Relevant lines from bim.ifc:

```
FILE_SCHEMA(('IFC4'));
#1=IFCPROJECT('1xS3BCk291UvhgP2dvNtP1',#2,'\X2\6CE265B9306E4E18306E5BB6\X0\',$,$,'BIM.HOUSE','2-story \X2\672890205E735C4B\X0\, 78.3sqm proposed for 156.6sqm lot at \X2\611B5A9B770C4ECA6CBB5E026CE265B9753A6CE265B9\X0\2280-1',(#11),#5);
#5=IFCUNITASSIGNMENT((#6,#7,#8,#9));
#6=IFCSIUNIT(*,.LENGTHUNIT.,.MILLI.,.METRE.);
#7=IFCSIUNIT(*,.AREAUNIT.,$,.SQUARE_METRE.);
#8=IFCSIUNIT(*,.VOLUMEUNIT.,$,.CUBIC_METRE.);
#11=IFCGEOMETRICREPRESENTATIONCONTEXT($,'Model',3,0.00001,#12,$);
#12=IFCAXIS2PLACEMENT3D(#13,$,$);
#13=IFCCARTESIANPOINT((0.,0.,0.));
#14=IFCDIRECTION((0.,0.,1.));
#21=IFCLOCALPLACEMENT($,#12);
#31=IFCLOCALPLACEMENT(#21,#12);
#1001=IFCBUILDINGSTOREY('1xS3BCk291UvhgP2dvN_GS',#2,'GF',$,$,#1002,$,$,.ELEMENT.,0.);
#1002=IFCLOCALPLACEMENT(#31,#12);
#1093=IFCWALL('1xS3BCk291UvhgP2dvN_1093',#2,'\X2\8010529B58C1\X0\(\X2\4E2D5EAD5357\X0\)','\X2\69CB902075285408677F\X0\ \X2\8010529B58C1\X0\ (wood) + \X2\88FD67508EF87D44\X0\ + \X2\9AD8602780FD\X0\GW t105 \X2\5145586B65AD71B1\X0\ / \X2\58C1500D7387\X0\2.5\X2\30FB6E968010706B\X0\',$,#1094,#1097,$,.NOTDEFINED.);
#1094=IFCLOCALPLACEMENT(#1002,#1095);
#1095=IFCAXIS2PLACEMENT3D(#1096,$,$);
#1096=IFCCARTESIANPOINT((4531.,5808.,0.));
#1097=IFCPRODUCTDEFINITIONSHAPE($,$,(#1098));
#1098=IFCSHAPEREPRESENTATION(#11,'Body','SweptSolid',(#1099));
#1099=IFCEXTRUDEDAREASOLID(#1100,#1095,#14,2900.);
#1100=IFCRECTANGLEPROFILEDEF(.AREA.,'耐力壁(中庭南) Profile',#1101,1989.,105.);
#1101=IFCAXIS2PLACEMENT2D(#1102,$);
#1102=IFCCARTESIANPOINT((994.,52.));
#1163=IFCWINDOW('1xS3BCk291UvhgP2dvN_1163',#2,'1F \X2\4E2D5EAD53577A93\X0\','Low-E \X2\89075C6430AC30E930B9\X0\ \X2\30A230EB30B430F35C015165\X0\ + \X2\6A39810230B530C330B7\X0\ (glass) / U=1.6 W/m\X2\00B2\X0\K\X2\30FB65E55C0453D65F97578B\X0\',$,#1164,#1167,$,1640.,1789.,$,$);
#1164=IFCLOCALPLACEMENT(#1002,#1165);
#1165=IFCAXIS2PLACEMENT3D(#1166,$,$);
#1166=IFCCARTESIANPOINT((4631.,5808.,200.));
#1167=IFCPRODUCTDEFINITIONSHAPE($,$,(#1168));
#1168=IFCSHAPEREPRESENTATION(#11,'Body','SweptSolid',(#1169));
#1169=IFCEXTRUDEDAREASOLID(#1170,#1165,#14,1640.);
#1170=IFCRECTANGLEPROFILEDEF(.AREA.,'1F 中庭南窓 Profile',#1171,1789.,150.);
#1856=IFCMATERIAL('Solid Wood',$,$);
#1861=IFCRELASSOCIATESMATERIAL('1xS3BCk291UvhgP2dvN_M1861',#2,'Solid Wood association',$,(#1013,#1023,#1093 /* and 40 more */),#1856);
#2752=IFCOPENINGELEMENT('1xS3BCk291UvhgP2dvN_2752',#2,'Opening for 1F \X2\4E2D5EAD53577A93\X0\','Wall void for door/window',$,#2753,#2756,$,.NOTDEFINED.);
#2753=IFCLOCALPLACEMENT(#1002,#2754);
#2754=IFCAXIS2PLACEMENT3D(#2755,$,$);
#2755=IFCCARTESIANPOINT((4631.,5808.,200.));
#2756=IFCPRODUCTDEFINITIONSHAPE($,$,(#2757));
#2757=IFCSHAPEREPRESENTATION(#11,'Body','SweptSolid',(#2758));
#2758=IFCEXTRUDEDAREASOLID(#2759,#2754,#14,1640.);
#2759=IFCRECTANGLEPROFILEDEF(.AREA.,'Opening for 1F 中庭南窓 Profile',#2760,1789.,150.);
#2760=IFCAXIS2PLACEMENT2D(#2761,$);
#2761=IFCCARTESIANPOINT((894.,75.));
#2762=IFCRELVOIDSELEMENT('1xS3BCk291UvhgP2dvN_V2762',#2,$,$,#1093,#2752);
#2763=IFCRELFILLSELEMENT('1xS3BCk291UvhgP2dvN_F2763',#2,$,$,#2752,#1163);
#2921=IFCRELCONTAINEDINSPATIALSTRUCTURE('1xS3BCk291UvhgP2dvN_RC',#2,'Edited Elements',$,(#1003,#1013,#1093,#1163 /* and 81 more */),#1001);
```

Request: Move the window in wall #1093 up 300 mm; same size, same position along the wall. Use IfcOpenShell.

```python
import numpy as np
import ifcopenshell
import ifcopenshell.api.geometry
import ifcopenshell.util.placement
import ifcopenshell.util.unit

model = ifcopenshell.open("bim.ifc")
unit_scale = ifcopenshell.util.unit.calculate_unit_scale(model)

window = model.by_guid("1xS3BCk291UvhgP2dvN_1163")
opening = window.FillsVoids[0].RelatingOpeningElement
dz = 0.3 / unit_scale

shift = np.array([0.0, 0.0, dz])
# The window is not placed relative to its opening, so move both.
for product in (opening, window):
    matrix = ifcopenshell.util.placement.get_local_placement(product.ObjectPlacement)
    matrix[:3, 3] += shift
    ifcopenshell.api.geometry.edit_object_placement(model, product=product, matrix=matrix, is_si=False)

print(f"moved by {dz * unit_scale:+.3f} m")

model.write("bim_rev.ifc")
```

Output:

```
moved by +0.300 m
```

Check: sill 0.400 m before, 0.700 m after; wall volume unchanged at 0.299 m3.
